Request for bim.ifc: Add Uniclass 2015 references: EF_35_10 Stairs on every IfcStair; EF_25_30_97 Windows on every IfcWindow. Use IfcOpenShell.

First a look at what the model holds.

```python
import ifcopenshell

model = ifcopenshell.open("bim.ifc")
print(model.schema)
print("classifications:", [c.Name for c in model.by_type("IfcClassification")])
for ifc_class in ("IfcDoor", "IfcRoof", "IfcStair", "IfcWall", "IfcWindow"):
    print(ifc_class, len(model.by_type(ifc_class)))
```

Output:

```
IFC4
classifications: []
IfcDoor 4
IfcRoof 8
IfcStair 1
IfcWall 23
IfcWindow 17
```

```python
import ifcopenshell
import ifcopenshell.api.classification

model = ifcopenshell.open("bim.ifc")

system = ifcopenshell.api.classification.add_classification(model, classification="Uniclass 2015")

codes = {
    "IfcStair": ("EF_35_10", "Stairs"),
    "IfcWindow": ("EF_25_30_97", "Windows"),
}
for ifc_class, (code, name) in codes.items():
    products = model.by_type(ifc_class)
    ifcopenshell.api.classification.add_reference(
        model, products=products, classification=system, identification=code, name=name
    )
    print(code, len(products))

model.write("bim_v2.ifc")
```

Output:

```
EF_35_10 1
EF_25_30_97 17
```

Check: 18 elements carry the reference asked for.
